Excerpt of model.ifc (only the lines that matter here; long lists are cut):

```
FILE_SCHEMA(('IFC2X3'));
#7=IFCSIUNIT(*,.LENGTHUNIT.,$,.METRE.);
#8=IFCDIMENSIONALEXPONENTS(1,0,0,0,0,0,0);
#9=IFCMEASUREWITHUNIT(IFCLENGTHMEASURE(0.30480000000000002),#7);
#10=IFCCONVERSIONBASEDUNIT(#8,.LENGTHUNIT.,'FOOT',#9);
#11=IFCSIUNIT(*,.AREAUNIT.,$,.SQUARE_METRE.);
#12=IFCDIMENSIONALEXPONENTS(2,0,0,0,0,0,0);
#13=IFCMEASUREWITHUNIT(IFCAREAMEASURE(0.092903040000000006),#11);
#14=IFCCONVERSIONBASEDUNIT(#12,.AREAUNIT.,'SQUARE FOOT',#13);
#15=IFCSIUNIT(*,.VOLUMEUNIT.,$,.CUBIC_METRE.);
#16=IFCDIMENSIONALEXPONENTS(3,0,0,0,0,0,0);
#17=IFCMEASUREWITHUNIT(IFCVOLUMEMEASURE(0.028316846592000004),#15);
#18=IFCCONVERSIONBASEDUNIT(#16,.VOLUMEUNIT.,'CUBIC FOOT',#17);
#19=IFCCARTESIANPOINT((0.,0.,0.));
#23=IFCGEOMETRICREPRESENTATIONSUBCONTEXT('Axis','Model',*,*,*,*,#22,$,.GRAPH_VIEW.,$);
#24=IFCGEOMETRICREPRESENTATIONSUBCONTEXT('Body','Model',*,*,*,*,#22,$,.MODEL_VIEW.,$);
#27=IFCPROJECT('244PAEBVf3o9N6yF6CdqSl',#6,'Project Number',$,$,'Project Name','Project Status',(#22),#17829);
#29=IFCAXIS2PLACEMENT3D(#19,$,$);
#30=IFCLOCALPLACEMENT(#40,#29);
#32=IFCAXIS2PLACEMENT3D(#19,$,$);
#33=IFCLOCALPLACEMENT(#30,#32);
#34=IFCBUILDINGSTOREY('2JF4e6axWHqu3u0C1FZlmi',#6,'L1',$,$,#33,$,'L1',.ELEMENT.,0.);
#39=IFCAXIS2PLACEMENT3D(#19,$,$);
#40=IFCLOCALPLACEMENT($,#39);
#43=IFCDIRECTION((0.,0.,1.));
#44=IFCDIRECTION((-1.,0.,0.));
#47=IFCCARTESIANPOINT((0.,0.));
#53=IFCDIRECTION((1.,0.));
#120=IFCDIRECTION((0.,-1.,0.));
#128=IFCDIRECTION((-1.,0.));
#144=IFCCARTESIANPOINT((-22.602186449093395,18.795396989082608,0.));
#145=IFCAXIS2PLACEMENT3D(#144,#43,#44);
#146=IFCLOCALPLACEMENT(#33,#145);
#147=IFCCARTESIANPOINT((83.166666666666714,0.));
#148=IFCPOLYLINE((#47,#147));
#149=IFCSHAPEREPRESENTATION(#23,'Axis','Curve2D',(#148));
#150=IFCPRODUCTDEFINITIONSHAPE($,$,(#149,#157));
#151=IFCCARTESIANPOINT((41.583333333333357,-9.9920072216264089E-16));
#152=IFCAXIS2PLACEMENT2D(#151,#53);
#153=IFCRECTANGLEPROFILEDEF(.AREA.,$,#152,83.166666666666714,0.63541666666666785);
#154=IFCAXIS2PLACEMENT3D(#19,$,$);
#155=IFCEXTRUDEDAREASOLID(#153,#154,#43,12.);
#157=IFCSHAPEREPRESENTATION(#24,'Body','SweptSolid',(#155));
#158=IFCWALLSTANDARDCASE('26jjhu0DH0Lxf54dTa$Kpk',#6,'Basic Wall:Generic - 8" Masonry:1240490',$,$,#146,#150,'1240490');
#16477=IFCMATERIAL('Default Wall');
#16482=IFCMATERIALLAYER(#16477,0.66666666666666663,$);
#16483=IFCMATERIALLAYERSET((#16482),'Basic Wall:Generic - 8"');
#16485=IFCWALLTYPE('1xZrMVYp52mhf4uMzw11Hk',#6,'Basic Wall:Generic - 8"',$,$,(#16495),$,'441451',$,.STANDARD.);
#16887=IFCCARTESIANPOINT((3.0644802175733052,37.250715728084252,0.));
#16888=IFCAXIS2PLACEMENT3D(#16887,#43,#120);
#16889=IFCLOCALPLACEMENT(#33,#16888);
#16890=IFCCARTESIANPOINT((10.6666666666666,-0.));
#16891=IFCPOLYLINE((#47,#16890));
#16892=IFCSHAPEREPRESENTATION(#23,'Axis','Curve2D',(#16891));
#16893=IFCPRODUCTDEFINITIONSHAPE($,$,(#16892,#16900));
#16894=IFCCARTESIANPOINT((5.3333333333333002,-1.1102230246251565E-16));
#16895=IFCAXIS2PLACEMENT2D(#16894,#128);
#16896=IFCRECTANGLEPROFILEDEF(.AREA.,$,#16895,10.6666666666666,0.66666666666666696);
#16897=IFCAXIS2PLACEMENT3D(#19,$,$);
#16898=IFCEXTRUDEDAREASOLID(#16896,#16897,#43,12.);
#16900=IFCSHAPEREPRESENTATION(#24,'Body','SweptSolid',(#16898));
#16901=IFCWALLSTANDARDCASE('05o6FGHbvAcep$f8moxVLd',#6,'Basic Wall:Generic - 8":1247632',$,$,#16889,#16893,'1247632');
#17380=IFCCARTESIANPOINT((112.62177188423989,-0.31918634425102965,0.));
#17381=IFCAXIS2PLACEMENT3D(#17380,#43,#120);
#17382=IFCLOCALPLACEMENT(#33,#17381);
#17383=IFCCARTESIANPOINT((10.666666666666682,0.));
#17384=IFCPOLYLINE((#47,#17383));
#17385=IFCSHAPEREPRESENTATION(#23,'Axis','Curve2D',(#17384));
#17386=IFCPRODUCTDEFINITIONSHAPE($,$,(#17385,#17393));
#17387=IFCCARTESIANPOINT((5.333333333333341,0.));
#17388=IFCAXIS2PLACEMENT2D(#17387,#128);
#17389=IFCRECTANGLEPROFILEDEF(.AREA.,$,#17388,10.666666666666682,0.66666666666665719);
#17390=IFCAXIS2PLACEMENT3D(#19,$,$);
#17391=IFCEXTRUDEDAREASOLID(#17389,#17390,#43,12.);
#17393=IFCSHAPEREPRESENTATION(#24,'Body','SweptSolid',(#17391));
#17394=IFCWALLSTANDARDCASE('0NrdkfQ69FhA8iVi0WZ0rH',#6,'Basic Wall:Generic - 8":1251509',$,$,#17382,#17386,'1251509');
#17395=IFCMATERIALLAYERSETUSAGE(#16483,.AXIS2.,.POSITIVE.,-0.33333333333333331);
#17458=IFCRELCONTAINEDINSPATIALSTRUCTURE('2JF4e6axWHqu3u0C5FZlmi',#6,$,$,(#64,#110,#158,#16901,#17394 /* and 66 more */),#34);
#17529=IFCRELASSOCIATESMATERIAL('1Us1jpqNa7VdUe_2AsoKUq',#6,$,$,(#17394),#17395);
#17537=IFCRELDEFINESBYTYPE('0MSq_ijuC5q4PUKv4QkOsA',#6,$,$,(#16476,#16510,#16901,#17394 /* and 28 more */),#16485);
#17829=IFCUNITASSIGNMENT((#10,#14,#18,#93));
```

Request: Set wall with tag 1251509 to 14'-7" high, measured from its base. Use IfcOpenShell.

```python
import ifcopenshell
import ifcopenshell.geom
import ifcopenshell.util.representation
import ifcopenshell.util.shape
import ifcopenshell.util.unit

model = ifcopenshell.open("model.ifc")
unit_scale = ifcopenshell.util.unit.calculate_unit_scale(model)
settings = ifcopenshell.geom.settings()


def volume(element):
    """Net volume in cubic metres, openings subtracted."""
    shape = ifcopenshell.geom.create_shape(settings, element)
    return ifcopenshell.util.shape.get_volume(shape.geometry)


wall = model.by_guid("0NrdkfQ69FhA8iVi0WZ0rH")
before = volume(wall)

body = ifcopenshell.util.representation.get_representation(wall, "Model", "Body")
solid = body.Items[0]
old_height = solid.Depth
solid.Depth = 175 * 0.0254 / unit_scale
after = volume(wall)

print(f"height {old_height:g} -> {solid.Depth:g}, volume {before:.3f} -> {after:.3f} m3")

model.write("model_v2.ifc")
```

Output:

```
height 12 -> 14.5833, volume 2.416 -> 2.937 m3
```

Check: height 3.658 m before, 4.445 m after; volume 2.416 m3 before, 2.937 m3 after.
